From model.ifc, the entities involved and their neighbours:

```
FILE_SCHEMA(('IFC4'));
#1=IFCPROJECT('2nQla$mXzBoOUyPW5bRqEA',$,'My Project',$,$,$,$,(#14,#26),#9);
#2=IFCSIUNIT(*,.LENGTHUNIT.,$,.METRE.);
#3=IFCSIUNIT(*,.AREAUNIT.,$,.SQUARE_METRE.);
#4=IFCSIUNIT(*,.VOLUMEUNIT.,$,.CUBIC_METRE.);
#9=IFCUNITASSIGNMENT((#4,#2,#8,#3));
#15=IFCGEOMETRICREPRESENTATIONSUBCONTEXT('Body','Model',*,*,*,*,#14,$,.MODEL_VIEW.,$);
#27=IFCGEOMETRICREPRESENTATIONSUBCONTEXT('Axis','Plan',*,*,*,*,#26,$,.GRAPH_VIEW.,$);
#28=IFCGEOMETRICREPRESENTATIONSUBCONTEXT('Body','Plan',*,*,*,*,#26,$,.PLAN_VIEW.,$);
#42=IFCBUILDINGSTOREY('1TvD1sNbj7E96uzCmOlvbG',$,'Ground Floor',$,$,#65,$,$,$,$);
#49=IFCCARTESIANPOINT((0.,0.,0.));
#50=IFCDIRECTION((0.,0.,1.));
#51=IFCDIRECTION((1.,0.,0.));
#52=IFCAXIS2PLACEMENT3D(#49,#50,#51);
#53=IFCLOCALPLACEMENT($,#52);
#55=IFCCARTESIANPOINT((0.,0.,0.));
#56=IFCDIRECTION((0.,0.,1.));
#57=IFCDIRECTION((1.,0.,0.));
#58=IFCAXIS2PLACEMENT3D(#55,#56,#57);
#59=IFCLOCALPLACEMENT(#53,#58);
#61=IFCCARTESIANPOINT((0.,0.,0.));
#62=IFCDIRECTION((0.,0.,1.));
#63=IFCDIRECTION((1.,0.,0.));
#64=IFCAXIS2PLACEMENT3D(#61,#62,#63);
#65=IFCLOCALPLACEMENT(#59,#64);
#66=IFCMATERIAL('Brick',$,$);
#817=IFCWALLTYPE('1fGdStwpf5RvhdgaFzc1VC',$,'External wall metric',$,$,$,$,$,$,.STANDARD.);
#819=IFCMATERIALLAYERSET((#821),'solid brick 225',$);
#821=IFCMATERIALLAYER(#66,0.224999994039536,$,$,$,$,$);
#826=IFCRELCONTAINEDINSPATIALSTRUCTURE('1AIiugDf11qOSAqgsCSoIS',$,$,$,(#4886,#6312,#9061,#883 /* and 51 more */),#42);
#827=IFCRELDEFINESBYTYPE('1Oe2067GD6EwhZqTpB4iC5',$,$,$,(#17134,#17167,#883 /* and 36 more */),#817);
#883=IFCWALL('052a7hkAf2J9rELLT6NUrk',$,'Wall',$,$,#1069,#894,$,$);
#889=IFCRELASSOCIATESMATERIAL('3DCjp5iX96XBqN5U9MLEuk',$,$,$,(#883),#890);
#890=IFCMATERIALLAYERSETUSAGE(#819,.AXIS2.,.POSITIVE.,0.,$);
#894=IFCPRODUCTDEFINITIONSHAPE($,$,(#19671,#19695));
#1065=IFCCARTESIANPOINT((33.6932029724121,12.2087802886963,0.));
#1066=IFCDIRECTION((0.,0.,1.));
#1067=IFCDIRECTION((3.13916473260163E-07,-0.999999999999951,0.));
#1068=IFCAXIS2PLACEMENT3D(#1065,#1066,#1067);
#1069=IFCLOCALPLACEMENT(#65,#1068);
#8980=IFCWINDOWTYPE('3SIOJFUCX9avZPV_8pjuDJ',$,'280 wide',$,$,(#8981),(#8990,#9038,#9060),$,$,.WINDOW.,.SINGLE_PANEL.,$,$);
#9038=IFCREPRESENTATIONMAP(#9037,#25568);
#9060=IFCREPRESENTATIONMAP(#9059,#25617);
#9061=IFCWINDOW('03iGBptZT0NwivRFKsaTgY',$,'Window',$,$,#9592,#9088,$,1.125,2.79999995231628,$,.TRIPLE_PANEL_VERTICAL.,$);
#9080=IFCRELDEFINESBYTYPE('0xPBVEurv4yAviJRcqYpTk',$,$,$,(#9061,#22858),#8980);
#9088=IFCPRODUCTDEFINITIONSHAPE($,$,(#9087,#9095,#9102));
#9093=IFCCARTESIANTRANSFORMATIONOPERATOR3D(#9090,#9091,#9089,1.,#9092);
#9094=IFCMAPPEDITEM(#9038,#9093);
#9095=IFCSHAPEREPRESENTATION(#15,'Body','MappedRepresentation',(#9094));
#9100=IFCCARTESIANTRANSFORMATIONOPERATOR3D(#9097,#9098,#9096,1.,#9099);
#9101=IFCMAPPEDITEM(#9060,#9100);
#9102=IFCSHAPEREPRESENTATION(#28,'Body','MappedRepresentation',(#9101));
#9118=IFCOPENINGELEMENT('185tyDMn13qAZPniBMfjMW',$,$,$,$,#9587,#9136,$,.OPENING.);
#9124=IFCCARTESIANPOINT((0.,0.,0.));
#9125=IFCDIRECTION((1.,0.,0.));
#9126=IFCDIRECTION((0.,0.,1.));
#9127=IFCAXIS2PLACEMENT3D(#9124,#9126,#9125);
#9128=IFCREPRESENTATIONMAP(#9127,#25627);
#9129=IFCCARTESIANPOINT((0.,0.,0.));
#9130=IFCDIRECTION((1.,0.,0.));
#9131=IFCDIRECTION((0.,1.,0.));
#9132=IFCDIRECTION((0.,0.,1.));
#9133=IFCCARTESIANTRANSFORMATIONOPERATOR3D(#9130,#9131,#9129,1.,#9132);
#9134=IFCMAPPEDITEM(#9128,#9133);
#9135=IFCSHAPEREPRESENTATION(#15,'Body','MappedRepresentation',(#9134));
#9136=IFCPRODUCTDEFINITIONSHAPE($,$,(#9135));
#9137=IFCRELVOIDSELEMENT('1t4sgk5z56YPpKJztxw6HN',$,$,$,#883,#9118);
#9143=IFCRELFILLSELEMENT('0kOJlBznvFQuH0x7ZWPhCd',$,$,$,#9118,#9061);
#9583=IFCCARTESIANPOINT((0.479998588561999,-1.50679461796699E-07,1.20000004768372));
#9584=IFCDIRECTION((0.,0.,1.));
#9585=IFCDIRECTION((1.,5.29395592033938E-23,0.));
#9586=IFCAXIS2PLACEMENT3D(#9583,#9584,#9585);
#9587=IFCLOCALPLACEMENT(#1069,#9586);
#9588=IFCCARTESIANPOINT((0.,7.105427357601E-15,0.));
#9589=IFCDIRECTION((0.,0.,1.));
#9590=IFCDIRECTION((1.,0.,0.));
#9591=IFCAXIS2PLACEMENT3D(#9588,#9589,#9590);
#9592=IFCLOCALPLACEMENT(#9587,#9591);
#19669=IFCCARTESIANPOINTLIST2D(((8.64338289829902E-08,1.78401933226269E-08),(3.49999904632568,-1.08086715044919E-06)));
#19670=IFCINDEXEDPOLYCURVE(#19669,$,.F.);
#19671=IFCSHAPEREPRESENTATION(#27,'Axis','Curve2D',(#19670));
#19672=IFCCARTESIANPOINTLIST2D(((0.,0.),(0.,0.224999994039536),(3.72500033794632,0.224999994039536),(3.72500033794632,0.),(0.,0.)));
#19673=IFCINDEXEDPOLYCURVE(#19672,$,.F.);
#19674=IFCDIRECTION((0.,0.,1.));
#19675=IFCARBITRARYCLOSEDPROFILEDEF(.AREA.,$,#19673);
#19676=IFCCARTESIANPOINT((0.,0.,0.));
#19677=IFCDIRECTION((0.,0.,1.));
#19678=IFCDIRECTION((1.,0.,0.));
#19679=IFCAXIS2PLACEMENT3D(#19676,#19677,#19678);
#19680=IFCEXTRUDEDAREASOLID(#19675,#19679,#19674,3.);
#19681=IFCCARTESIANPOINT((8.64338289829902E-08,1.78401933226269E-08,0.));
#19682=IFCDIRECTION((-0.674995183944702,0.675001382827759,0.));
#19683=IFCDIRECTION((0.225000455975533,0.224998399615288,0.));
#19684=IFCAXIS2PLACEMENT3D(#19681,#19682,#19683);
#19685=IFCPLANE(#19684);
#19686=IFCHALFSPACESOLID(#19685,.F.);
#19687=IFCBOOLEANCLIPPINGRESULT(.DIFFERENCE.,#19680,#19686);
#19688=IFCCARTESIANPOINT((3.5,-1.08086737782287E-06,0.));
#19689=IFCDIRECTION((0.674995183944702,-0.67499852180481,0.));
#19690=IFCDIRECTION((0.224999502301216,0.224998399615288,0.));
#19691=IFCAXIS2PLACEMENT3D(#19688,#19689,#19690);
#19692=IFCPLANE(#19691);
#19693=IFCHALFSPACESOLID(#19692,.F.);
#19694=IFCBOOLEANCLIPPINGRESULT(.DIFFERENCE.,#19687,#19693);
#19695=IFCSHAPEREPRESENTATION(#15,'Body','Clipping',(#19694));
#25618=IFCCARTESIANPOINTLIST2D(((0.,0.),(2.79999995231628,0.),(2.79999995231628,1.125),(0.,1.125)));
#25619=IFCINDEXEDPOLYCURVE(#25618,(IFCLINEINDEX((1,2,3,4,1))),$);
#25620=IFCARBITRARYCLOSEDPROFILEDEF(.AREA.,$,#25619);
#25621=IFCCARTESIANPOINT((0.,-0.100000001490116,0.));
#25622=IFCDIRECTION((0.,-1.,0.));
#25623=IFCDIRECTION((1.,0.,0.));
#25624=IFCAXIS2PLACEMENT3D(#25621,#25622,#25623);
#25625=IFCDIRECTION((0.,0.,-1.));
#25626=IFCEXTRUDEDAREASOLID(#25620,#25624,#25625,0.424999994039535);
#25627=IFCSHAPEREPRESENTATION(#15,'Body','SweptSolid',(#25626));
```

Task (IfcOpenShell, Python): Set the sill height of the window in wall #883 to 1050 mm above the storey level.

```python
import numpy as np
import ifcopenshell
import ifcopenshell.api.geometry
import ifcopenshell.geom
import ifcopenshell.util.element
import ifcopenshell.util.placement
import ifcopenshell.util.shape
import ifcopenshell.util.unit

model = ifcopenshell.open("model.ifc")
unit_scale = ifcopenshell.util.unit.calculate_unit_scale(model)

window = model.by_id(9061)
opening = window.FillsVoids[0].RelatingOpeningElement
storey = ifcopenshell.util.element.get_container(window, ifc_class="IfcBuildingStorey")
level = ifcopenshell.util.placement.get_local_placement(storey.ObjectPlacement)[2, 3]

# The opening's origin need not be at the sill, so measure its lowest point.
shape = ifcopenshell.geom.create_shape(ifcopenshell.geom.settings(), opening)
bottom = ifcopenshell.util.shape.get_shape_bottom_elevation(shape, shape.geometry) / unit_scale
dz = level + 1.05 / unit_scale - bottom

shift = np.array([0.0, 0.0, dz])
# The window is placed relative to its opening, so it follows when the opening moves.
matrix = ifcopenshell.util.placement.get_local_placement(opening.ObjectPlacement)
matrix[:3, 3] += shift
ifcopenshell.api.geometry.edit_object_placement(
    model, product=opening, matrix=matrix, is_si=False, should_transform_children=True
)

print(f"moved by {dz * unit_scale:+.3f} m")

model.write("model_updated.ifc")
```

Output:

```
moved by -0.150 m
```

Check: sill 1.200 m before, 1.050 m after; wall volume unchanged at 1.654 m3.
